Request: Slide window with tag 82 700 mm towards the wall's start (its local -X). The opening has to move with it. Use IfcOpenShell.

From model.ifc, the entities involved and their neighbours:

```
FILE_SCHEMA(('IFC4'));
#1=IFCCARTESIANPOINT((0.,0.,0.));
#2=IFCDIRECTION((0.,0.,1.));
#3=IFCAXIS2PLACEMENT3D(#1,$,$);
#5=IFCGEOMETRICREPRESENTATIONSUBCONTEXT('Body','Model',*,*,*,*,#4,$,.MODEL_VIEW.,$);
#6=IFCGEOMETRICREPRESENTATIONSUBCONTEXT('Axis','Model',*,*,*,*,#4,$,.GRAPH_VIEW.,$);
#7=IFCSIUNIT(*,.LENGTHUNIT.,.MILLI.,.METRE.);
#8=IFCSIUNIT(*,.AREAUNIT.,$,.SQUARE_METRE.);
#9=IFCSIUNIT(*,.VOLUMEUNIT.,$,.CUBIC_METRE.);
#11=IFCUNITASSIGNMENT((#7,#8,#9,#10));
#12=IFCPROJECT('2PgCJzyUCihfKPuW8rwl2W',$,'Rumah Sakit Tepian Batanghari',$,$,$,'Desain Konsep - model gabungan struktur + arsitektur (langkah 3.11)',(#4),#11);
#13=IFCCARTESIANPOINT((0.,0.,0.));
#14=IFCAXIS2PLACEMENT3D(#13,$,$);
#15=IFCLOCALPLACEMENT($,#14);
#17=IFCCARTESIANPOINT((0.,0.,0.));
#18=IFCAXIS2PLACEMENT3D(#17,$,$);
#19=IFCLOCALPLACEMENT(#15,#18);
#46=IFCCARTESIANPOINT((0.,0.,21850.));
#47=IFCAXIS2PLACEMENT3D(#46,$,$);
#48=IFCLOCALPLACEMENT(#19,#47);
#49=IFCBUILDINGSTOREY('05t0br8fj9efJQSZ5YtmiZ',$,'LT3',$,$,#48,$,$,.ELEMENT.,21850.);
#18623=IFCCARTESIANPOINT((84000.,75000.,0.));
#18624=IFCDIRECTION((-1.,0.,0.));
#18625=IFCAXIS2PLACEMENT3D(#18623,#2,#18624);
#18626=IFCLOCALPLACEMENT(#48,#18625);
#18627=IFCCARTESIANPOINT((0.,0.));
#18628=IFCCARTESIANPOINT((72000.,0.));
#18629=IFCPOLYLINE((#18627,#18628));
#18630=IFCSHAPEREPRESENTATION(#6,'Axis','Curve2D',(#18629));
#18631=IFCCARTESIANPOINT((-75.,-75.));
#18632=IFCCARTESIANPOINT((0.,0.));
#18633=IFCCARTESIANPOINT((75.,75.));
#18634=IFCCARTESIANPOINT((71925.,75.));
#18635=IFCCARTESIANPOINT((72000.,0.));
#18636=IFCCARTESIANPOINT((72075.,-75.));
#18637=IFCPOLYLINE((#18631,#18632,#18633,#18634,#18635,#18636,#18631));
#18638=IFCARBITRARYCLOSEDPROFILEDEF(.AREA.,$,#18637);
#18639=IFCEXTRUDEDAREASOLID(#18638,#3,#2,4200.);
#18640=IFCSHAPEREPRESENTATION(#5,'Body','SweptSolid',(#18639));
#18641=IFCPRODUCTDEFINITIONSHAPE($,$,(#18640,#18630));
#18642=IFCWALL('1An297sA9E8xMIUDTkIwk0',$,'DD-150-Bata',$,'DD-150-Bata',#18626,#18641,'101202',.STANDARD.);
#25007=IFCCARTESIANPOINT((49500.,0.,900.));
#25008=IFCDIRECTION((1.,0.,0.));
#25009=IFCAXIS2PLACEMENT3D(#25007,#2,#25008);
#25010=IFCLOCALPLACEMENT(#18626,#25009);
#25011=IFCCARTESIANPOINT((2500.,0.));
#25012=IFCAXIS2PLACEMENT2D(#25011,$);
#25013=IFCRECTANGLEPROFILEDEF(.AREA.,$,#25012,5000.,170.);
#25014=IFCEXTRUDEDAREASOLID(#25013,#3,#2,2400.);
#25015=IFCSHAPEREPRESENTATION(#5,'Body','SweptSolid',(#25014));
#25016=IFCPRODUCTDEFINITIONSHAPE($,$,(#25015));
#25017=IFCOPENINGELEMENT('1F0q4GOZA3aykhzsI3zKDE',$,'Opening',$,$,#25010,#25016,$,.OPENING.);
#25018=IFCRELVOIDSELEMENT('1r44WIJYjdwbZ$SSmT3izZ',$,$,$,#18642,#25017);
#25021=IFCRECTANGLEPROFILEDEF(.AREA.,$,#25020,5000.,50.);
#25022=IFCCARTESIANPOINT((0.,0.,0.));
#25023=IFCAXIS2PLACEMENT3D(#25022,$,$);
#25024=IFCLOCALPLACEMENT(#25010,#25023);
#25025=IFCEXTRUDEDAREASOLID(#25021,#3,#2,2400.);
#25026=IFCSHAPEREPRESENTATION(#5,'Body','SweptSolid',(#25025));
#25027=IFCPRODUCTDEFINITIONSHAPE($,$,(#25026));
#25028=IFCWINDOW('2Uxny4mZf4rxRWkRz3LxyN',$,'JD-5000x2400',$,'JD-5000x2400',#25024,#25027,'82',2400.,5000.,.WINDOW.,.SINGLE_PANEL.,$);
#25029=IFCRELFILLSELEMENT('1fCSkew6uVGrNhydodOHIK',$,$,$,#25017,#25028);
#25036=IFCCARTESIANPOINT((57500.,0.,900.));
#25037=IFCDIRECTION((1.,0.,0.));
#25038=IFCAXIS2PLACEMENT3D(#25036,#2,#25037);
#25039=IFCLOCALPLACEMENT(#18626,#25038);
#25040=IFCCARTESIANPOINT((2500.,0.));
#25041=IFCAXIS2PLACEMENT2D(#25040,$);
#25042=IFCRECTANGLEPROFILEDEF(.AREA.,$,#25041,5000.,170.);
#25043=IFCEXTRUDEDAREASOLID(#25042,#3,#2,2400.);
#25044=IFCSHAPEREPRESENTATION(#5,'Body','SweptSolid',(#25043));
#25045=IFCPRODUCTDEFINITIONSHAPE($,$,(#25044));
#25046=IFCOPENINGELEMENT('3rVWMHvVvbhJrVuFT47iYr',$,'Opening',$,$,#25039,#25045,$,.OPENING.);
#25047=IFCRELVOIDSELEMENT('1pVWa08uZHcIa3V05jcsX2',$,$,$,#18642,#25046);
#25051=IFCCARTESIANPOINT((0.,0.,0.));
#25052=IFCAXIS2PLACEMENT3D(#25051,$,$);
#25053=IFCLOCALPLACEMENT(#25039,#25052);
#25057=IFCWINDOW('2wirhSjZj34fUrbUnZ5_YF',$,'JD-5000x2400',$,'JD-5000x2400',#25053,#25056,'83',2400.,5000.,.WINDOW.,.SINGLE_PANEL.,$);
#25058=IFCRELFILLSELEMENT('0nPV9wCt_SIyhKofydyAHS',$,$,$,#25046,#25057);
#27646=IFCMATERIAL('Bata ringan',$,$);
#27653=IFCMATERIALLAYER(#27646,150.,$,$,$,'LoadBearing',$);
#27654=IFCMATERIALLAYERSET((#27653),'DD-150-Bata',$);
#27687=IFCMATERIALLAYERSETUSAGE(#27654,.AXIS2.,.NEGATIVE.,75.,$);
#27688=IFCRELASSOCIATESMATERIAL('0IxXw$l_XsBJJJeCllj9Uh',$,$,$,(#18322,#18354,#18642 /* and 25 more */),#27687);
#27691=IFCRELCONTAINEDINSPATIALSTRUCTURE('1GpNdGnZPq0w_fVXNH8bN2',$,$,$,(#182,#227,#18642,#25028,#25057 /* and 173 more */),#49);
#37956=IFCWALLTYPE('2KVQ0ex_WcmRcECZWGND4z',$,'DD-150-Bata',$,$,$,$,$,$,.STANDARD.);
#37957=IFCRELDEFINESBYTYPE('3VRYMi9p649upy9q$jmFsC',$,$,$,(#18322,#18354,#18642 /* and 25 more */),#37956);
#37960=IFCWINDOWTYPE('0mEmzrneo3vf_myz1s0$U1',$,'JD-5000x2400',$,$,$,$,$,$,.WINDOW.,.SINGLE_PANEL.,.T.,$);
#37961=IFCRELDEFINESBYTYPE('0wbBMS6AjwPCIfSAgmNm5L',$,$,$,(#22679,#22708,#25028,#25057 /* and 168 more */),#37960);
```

```python
import ifcopenshell
import ifcopenshell.api.geometry
import ifcopenshell.util.placement

model = ifcopenshell.open("model.ifc")

window = model.by_id(25028)
opening = window.FillsVoids[0].RelatingOpeningElement
wall = opening.VoidsElements[0].RelatingBuildingElement

wall_matrix = ifcopenshell.util.placement.get_local_placement(wall.ObjectPlacement)
shift = wall_matrix[:3, 0] * -700.0
before = ifcopenshell.util.placement.get_local_placement(window.ObjectPlacement)[:3, 3].copy()

# The window is placed relative to its opening, so it follows when the opening moves.
matrix = ifcopenshell.util.placement.get_local_placement(opening.ObjectPlacement)
matrix[:3, 3] += shift
ifcopenshell.api.geometry.edit_object_placement(
    model, product=opening, matrix=matrix, is_si=False, should_transform_children=True
)

after = ifcopenshell.util.placement.get_local_placement(window.ObjectPlacement)[:3, 3]
print("window moved by", (after - before).round(3) + 0.0)

model.write("model-out.ifc")
```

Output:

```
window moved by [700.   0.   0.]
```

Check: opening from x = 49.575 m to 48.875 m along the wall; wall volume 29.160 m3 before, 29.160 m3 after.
